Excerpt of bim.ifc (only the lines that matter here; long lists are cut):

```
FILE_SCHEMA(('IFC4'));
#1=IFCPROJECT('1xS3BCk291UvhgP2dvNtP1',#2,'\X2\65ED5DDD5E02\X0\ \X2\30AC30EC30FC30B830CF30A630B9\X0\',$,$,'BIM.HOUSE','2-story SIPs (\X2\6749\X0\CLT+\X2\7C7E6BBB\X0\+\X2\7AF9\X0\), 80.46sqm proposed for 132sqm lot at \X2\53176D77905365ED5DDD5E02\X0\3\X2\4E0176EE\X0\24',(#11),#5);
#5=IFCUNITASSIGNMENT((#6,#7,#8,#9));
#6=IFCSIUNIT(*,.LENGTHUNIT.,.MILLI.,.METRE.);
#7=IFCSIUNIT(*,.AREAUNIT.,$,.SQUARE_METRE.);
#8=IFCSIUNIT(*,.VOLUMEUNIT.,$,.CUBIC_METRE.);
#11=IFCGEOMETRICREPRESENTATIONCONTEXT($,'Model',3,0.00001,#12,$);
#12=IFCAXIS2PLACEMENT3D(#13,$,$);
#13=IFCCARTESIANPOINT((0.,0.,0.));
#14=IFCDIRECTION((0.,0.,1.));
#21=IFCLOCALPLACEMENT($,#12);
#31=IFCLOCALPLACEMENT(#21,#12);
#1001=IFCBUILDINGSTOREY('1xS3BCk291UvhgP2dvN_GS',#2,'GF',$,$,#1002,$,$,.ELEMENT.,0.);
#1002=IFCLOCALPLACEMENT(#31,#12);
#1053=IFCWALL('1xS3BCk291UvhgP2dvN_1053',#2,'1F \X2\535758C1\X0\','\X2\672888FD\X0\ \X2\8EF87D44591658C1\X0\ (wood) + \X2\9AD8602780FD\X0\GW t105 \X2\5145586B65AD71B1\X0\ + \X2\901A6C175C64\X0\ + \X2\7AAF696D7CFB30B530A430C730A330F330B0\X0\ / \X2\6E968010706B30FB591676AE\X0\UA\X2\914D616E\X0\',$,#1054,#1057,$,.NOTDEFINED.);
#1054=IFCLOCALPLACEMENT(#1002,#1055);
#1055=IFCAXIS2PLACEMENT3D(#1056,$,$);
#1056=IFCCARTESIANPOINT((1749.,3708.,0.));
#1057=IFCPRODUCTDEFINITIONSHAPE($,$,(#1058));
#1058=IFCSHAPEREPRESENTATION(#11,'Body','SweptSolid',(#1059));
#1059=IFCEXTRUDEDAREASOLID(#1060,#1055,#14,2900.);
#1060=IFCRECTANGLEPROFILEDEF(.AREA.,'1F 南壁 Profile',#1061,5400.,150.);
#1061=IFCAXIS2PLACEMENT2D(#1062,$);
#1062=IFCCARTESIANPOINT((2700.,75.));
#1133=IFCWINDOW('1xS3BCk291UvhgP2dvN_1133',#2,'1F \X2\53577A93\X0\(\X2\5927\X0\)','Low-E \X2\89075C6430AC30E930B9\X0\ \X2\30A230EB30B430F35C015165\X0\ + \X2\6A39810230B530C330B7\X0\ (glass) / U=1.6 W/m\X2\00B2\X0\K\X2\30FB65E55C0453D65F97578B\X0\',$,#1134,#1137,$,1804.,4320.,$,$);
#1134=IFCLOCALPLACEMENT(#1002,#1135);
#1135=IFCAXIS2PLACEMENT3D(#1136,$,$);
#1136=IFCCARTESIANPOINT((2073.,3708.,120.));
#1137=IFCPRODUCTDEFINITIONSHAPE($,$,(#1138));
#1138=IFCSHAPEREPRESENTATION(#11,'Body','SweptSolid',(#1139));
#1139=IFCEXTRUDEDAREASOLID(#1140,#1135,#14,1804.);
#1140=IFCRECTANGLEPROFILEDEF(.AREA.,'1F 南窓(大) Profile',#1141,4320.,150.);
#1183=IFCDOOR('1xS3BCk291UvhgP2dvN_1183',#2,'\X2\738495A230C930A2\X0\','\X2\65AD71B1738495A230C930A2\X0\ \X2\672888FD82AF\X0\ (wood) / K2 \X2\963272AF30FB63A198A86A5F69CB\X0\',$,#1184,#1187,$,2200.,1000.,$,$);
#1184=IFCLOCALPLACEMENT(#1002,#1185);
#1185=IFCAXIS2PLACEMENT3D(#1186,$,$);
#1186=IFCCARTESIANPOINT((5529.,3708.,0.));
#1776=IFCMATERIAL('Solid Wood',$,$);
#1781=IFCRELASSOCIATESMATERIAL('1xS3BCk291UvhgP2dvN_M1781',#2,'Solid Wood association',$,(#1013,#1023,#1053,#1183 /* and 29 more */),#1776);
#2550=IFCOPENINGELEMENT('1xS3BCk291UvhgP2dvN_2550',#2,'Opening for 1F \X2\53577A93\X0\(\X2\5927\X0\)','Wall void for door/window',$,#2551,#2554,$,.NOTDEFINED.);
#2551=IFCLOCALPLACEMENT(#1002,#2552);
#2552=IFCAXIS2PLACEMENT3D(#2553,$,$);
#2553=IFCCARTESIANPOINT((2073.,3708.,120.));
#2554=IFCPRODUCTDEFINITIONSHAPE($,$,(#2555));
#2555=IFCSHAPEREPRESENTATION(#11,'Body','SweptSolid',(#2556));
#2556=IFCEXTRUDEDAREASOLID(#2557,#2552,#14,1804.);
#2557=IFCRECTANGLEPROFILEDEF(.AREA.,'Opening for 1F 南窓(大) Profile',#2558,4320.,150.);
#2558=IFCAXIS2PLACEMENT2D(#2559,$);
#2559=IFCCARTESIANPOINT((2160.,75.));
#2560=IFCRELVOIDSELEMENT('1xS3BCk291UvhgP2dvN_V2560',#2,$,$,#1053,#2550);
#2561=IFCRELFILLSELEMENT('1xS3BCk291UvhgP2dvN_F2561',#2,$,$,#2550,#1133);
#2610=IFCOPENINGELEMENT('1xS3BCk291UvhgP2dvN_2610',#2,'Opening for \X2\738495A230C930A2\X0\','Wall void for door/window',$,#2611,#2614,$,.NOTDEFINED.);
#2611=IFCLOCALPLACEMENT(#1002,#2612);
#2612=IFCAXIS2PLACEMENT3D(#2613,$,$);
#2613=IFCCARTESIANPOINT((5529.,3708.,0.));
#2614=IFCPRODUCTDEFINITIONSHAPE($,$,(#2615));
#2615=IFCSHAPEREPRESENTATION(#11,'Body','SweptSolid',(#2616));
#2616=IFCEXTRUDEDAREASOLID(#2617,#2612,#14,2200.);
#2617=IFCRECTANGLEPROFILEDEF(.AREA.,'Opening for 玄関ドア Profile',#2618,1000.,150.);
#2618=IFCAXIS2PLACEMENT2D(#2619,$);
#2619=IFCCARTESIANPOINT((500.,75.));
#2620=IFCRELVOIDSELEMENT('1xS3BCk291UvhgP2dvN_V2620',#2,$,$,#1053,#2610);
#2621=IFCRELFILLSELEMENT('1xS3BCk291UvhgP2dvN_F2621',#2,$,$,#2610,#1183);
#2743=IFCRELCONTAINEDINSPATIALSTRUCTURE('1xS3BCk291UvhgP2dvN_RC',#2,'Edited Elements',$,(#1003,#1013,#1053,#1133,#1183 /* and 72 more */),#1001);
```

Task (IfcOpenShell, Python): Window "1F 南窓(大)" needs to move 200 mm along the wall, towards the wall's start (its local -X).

```python
import ifcopenshell
import ifcopenshell.api.geometry
import ifcopenshell.util.placement
import ifcopenshell.util.unit

model = ifcopenshell.open("bim.ifc")
unit_scale = ifcopenshell.util.unit.calculate_unit_scale(model)

window = model.by_id(1133)
opening = window.FillsVoids[0].RelatingOpeningElement
wall = opening.VoidsElements[0].RelatingBuildingElement

wall_matrix = ifcopenshell.util.placement.get_local_placement(wall.ObjectPlacement)
shift = wall_matrix[:3, 0] * -0.2 / unit_scale
before = ifcopenshell.util.placement.get_local_placement(window.ObjectPlacement)[:3, 3].copy()

# The window is not placed relative to its opening, so move both.
for product in (opening, window):
    matrix = ifcopenshell.util.placement.get_local_placement(product.ObjectPlacement)
    matrix[:3, 3] += shift
    ifcopenshell.api.geometry.edit_object_placement(model, product=product, matrix=matrix, is_si=False)

after = ifcopenshell.util.placement.get_local_placement(window.ObjectPlacement)[:3, 3]
print("window moved by", (after - before).round(3) + 0.0)

model.write("bim_updated.ifc")
```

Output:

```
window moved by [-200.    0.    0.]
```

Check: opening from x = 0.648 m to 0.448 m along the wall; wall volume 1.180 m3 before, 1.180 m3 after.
